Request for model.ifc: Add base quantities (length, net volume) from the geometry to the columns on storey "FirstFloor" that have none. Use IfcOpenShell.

First a look at what the model holds.

```python
import ifcopenshell
import ifcopenshell.util.element
import ifcopenshell.util.unit

model = ifcopenshell.open("model.ifc")
print(model.schema)
for unit_type in ("LENGTHUNIT", "AREAUNIT", "VOLUMEUNIT"):
    print(unit_type, ifcopenshell.util.unit.calculate_unit_scale(model, unit_type))
storey = next(s for s in model.by_type("IfcBuildingStorey") if s.Name == "FirstFloor")
columns = [e for e in ifcopenshell.util.element.get_decomposition(storey) if e.is_a("IfcColumn")]
for e in sorted(columns, key=lambda e: e.id()):
    print(e.id(), e.is_a(), e.Name, list(ifcopenshell.util.element.get_psets(e, qtos_only=True)), sep=" | ")
```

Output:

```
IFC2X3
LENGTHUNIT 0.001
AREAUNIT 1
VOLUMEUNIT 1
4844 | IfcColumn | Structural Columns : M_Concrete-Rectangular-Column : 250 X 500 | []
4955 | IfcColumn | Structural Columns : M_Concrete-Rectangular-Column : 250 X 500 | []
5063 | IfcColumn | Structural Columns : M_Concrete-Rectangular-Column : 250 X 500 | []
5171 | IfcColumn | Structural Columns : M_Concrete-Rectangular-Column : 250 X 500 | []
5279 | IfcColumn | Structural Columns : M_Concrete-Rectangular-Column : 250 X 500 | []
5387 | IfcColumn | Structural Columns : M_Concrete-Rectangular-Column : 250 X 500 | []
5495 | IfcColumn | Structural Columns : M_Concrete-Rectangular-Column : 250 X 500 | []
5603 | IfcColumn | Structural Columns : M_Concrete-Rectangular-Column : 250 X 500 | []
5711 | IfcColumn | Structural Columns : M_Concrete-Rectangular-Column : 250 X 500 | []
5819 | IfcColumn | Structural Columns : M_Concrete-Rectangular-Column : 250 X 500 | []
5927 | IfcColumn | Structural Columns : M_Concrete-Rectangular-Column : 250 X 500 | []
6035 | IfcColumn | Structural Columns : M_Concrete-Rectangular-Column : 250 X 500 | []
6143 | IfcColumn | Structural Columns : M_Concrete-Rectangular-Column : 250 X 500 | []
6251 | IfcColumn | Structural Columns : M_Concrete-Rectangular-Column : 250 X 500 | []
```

```python
import ifcopenshell
import ifcopenshell.api.pset
import ifcopenshell.geom
import ifcopenshell.util.element
import ifcopenshell.util.shape
import ifcopenshell.util.unit

model = ifcopenshell.open("model.ifc")
unit_scale = ifcopenshell.util.unit.calculate_unit_scale(model)
volume_scale = ifcopenshell.util.unit.calculate_unit_scale(model, "VOLUMEUNIT")
settings = ifcopenshell.geom.settings()

storey = next(s for s in model.by_type("IfcBuildingStorey") if s.Name == "FirstFloor")
columns = [e for e in ifcopenshell.util.element.get_decomposition(storey) if e.is_a("IfcColumn")]

for e in sorted(columns, key=lambda e: e.id()):
    if ifcopenshell.util.element.get_psets(e, qtos_only=True, should_inherit=False):
        continue
    # Geometry comes back in metres, in the element's own axes.
    shape = ifcopenshell.geom.create_shape(settings, e)
    values = {
        "Length": ifcopenshell.util.shape.get_z(shape.geometry) / unit_scale,
        "NetVolume": ifcopenshell.util.shape.get_volume(shape.geometry) / volume_scale,
    }
    qto = ifcopenshell.api.pset.add_qto(model, product=e, name="BaseQuantities")
    ifcopenshell.api.pset.edit_qto(model, qto=qto, properties=values)
    print(e.id(), {k: round(v, 3) for k, v in values.items()})

model.write("model_v2.ifc")
```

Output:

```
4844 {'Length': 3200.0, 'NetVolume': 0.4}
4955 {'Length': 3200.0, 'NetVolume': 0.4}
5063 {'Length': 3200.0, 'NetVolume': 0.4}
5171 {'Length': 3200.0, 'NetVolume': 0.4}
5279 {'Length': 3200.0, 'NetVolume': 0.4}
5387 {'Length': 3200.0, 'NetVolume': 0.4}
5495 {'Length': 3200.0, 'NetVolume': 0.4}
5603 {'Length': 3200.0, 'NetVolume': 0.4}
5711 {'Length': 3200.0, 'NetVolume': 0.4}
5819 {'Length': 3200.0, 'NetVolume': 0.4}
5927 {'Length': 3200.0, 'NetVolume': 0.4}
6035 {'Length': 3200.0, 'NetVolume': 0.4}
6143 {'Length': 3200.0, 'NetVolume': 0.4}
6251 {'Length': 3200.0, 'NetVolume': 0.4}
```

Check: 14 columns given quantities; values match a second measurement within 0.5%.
